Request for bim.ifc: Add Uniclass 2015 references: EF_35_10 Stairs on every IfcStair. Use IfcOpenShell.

First a look at what the model holds.

```python
import ifcopenshell

model = ifcopenshell.open("bim.ifc")
print(model.schema)
print("classifications:", [c.Name for c in model.by_type("IfcClassification")])
for ifc_class in ("IfcDoor", "IfcRoof", "IfcStair", "IfcWall", "IfcWindow"):
    print(ifc_class, len(model.by_type(ifc_class)))
```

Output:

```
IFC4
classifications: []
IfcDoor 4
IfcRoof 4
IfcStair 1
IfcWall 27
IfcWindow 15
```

```python
import ifcopenshell
import ifcopenshell.api.classification

model = ifcopenshell.open("bim.ifc")

system = ifcopenshell.api.classification.add_classification(model, classification="Uniclass 2015")

codes = {
    "IfcStair": ("EF_35_10", "Stairs"),
}
for ifc_class, (code, name) in codes.items():
    products = model.by_type(ifc_class)
    ifcopenshell.api.classification.add_reference(
        model, products=products, classification=system, identification=code, name=name
    )
    print(code, len(products))

model.write("bim_rev.ifc")
```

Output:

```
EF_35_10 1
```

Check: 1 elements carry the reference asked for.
